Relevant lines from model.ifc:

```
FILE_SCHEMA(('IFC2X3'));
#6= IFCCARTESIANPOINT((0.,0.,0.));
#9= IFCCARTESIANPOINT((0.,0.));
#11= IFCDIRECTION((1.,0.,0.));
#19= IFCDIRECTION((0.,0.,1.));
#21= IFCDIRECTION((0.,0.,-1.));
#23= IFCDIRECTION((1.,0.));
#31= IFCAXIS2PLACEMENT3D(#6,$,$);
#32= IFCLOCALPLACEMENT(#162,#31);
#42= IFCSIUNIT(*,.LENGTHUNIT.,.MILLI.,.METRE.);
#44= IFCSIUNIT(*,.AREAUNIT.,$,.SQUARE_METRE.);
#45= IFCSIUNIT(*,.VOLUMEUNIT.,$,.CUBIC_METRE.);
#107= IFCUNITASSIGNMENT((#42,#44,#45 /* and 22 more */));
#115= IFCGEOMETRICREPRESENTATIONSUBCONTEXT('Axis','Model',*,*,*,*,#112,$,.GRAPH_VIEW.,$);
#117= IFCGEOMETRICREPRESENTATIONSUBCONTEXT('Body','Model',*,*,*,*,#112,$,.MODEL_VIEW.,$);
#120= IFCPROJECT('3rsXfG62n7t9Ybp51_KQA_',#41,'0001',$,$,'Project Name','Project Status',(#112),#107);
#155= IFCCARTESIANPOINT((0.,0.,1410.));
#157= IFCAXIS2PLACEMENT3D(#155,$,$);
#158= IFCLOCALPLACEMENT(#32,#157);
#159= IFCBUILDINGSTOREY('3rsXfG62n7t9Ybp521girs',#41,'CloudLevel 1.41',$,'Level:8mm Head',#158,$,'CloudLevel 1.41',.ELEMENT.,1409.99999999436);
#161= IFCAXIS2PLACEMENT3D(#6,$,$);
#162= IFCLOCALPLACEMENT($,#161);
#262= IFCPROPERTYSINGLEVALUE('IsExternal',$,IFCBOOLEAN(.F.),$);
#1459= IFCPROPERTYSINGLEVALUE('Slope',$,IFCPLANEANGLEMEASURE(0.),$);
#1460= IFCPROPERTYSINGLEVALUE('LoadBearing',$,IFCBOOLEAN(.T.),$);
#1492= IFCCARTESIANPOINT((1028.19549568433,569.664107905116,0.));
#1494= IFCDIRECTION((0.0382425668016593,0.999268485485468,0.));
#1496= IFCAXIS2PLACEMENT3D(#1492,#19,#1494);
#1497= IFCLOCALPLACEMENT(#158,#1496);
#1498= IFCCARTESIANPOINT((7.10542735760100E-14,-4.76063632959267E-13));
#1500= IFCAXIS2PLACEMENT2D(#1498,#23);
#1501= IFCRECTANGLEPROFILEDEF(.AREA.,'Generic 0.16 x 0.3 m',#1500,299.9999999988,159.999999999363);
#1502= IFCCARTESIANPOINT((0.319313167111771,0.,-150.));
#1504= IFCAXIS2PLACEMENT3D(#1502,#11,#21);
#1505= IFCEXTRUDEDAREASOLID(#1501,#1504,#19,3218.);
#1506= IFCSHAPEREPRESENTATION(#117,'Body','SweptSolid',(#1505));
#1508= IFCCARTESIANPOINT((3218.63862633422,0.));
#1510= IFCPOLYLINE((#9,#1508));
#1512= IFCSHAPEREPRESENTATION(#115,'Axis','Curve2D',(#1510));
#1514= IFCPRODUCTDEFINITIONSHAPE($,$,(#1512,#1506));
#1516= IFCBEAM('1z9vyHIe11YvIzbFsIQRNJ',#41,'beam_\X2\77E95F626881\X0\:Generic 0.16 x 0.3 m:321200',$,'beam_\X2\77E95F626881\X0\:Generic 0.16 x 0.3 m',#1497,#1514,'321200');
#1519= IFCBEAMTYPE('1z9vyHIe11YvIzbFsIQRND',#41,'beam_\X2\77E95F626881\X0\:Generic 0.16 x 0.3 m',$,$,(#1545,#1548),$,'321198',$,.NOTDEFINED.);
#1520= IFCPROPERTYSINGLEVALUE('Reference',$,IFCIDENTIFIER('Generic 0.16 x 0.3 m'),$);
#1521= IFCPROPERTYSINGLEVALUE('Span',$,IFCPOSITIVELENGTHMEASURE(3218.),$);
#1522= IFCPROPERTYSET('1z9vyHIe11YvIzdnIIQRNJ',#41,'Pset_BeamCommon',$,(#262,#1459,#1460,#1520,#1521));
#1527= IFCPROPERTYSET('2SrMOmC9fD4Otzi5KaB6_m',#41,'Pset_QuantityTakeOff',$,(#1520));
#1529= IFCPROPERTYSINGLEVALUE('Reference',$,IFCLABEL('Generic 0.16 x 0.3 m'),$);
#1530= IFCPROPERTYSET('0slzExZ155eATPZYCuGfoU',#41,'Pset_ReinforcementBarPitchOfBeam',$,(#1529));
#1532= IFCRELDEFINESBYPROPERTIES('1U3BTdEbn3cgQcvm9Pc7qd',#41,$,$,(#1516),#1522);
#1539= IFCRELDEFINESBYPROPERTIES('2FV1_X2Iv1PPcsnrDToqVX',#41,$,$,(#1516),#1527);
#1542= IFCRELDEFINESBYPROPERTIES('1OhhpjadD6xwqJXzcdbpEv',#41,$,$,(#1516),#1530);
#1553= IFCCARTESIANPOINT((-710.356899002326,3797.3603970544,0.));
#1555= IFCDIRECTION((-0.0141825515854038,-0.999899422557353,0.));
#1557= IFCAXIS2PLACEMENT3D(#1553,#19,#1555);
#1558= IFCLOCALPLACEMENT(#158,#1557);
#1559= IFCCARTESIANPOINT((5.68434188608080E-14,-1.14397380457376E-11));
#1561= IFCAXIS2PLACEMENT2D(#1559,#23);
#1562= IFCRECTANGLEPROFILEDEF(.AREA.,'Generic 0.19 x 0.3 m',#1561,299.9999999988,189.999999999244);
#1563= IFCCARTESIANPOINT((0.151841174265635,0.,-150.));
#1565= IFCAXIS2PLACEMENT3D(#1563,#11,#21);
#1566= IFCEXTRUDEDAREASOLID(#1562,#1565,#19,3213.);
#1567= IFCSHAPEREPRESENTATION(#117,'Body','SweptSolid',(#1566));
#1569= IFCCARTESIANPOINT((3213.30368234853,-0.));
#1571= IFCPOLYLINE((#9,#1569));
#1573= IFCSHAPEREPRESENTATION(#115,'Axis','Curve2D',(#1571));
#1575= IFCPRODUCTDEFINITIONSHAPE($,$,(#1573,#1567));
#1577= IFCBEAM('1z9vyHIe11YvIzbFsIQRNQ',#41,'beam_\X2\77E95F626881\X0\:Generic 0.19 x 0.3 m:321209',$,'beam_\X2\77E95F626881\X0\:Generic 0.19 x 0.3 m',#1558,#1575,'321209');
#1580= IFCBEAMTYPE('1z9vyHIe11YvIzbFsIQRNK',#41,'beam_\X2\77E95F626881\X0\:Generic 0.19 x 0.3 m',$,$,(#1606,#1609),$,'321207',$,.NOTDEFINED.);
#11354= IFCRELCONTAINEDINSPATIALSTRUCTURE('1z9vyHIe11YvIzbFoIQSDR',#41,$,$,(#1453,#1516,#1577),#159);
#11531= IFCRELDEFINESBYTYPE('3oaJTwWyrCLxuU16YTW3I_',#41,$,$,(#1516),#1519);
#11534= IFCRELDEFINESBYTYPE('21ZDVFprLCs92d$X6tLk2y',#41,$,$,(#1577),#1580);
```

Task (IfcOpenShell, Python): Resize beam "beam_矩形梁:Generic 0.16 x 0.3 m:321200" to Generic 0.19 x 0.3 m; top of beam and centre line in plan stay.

```python
import ifcopenshell
import ifcopenshell.api.pset
import ifcopenshell.api.type
import ifcopenshell.util.element
import ifcopenshell.util.representation

model = ifcopenshell.open("model.ifc")

member = model.by_guid("1z9vyHIe11YvIzbFsIQRNJ")
source = next(p for p in model.by_type("IfcRectangleProfileDef") if p.ProfileName == "Generic 0.19 x 0.3 m")

body = ifcopenshell.util.representation.get_representation(member, "Model", "Body")
solid = body.Items[0]
old_profile = solid.SweptArea

# Copy the section's sizes but keep this member's own profile position.
profile = ifcopenshell.util.element.copy(model, source)
# Profiles are centred, so shift by half the change in depth to hold the top.
shift = (old_profile.XDim - profile.XDim) / 2
x, y = old_profile.Position.Location.Coordinates
up = (-1.0, 0.0)  # upwards, in the solid's own plane
location = model.createIfcCartesianPoint((x + up[0] * shift, y + up[1] * shift))
profile.Position = model.createIfcAxis2Placement2D(location, old_profile.Position.RefDirection)
solid.SweptArea = profile
if not model.get_total_inverses(old_profile):
    ifcopenshell.util.element.remove_deep2(model, old_profile)

new_type = model.by_guid("1z9vyHIe11YvIzbFsIQRNK")
ifcopenshell.api.type.assign_type(
    model, related_objects=[member], relating_type=new_type, should_map_representations=False
)
member.Name = member.Name.replace("Generic 0.16 x 0.3 m", "Generic 0.19 x 0.3 m")
member.ObjectType = "beam_矩形梁:Generic 0.19 x 0.3 m"
pset = model.by_id(ifcopenshell.util.element.get_pset(member, "Pset_BeamCommon", should_inherit=False)["id"])
ifcopenshell.api.pset.edit_pset(model, pset=pset, properties={"Reference": "Generic 0.19 x 0.3 m"})
pset = model.by_id(ifcopenshell.util.element.get_pset(member, "Pset_QuantityTakeOff", should_inherit=False)["id"])
ifcopenshell.api.pset.edit_pset(model, pset=pset, properties={"Reference": "Generic 0.19 x 0.3 m"})
pset = model.by_id(ifcopenshell.util.element.get_pset(member, "Pset_ReinforcementBarPitchOfBeam", should_inherit=False)["id"])
ifcopenshell.api.pset.edit_pset(model, pset=pset, properties={"Reference": "Generic 0.19 x 0.3 m"})

print(solid.SweptArea)

model.write("model_rev.ifc")
```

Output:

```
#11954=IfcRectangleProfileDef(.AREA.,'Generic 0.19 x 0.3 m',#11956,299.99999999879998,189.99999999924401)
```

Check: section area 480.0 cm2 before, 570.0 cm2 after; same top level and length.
